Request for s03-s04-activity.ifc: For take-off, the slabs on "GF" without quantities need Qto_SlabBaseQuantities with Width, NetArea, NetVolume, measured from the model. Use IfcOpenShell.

First a look at what the model holds.

```python
import ifcopenshell
import ifcopenshell.util.element
import ifcopenshell.util.unit

model = ifcopenshell.open("s03-s04-activity.ifc")
print(model.schema)
for unit_type in ("LENGTHUNIT", "AREAUNIT", "VOLUMEUNIT"):
    print(unit_type, ifcopenshell.util.unit.calculate_unit_scale(model, unit_type))
storey = next(s for s in model.by_type("IfcBuildingStorey") if s.Name == "GF")
slabs = [e for e in ifcopenshell.util.element.get_decomposition(storey) if e.is_a("IfcSlab")]
for e in sorted(slabs, key=lambda e: e.id()):
    print(e.id(), e.is_a(), e.Name, list(ifcopenshell.util.element.get_psets(e, qtos_only=True)), sep=" | ")
```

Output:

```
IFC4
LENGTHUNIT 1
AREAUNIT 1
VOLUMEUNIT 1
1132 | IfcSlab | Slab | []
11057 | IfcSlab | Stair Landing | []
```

```python
import ifcopenshell
import ifcopenshell.api.pset
import ifcopenshell.geom
import ifcopenshell.util.element
import ifcopenshell.util.shape
import ifcopenshell.util.unit

model = ifcopenshell.open("s03-s04-activity.ifc")
unit_scale = ifcopenshell.util.unit.calculate_unit_scale(model)
area_scale = ifcopenshell.util.unit.calculate_unit_scale(model, "AREAUNIT")
volume_scale = ifcopenshell.util.unit.calculate_unit_scale(model, "VOLUMEUNIT")
settings = ifcopenshell.geom.settings()

storey = next(s for s in model.by_type("IfcBuildingStorey") if s.Name == "GF")
slabs = [e for e in ifcopenshell.util.element.get_decomposition(storey) if e.is_a("IfcSlab")]

for e in sorted(slabs, key=lambda e: e.id()):
    if ifcopenshell.util.element.get_psets(e, qtos_only=True, should_inherit=False):
        continue
    # Geometry comes back in metres, in the element's own axes.
    shape = ifcopenshell.geom.create_shape(settings, e)
    values = {
        "Width": ifcopenshell.util.shape.get_z(shape.geometry) / unit_scale,
        "NetArea": ifcopenshell.util.shape.get_footprint_area(shape.geometry) / area_scale,
        "NetVolume": ifcopenshell.util.shape.get_volume(shape.geometry) / volume_scale,
    }
    qto = ifcopenshell.api.pset.add_qto(model, product=e, name="Qto_SlabBaseQuantities")
    ifcopenshell.api.pset.edit_qto(model, qto=qto, properties=values)
    print(e.id(), {k: round(v, 3) for k, v in values.items()})

model.write("s03-s04-activity_rev.ifc")
```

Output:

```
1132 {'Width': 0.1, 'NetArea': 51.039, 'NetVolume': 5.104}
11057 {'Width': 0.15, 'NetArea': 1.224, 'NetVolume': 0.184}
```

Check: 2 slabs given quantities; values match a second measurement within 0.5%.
